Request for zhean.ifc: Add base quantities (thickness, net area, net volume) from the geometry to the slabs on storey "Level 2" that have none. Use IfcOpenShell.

First a look at what the model holds.

```python
import ifcopenshell
import ifcopenshell.util.element
import ifcopenshell.util.unit

model = ifcopenshell.open("zhean.ifc")
print(model.schema)
for unit_type in ("LENGTHUNIT", "AREAUNIT", "VOLUMEUNIT"):
    print(unit_type, ifcopenshell.util.unit.calculate_unit_scale(model, unit_type))
storey = next(s for s in model.by_type("IfcBuildingStorey") if s.Name == "Level 2")
slabs = [e for e in ifcopenshell.util.element.get_decomposition(storey) if e.is_a("IfcSlab")]
for e in sorted(slabs, key=lambda e: e.id()):
    print(e.id(), e.is_a(), e.Name, list(ifcopenshell.util.element.get_psets(e, qtos_only=True)), sep=" | ")
```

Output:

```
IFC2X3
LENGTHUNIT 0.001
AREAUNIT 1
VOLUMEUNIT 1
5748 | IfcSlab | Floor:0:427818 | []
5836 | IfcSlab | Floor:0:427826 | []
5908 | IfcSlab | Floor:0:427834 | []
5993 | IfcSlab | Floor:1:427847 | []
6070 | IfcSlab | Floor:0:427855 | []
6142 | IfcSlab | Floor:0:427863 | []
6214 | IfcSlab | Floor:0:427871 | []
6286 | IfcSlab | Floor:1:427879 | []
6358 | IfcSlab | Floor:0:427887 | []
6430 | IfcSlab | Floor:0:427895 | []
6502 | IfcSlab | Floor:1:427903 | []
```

```python
import ifcopenshell
import ifcopenshell.api.pset
import ifcopenshell.geom
import ifcopenshell.util.element
import ifcopenshell.util.shape
import ifcopenshell.util.unit

model = ifcopenshell.open("zhean.ifc")
unit_scale = ifcopenshell.util.unit.calculate_unit_scale(model)
area_scale = ifcopenshell.util.unit.calculate_unit_scale(model, "AREAUNIT")
volume_scale = ifcopenshell.util.unit.calculate_unit_scale(model, "VOLUMEUNIT")
settings = ifcopenshell.geom.settings()

storey = next(s for s in model.by_type("IfcBuildingStorey") if s.Name == "Level 2")
slabs = [e for e in ifcopenshell.util.element.get_decomposition(storey) if e.is_a("IfcSlab")]

for e in sorted(slabs, key=lambda e: e.id()):
    if ifcopenshell.util.element.get_psets(e, qtos_only=True, should_inherit=False):
        continue
    # Geometry comes back in metres, in the element's own axes.
    shape = ifcopenshell.geom.create_shape(settings, e)
    values = {
        "Width": ifcopenshell.util.shape.get_z(shape.geometry) / unit_scale,
        "NetArea": ifcopenshell.util.shape.get_footprint_area(shape.geometry) / area_scale,
        "NetVolume": ifcopenshell.util.shape.get_volume(shape.geometry) / volume_scale,
    }
    qto = ifcopenshell.api.pset.add_qto(model, product=e, name="BaseQuantities")
    ifcopenshell.api.pset.edit_qto(model, qto=qto, properties=values)
    print(e.id(), {k: round(v, 3) for k, v in values.items()})

model.write("zhean_edited.ifc")
```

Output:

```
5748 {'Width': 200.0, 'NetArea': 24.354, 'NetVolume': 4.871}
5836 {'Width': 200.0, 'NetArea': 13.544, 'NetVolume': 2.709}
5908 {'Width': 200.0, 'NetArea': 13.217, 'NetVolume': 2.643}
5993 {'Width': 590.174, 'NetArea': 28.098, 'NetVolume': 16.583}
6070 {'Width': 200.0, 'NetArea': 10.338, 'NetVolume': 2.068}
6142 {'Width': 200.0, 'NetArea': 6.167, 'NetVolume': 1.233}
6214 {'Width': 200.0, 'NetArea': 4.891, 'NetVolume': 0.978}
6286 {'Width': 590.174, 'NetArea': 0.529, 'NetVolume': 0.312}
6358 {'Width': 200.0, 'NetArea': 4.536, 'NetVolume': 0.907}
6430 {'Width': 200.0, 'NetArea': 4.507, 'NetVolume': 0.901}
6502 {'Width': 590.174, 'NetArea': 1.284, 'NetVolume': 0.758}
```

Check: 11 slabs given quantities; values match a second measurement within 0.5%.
